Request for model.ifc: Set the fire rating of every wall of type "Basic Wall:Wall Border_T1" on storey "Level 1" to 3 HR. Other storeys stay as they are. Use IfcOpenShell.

First a look at what the model holds.

```python
import ifcopenshell
import ifcopenshell.util.element

model = ifcopenshell.open("model.ifc")
print(model.schema)
storey = next(s for s in model.by_type("IfcBuildingStorey") if s.Name == "Level 1")
walls = [e for e in ifcopenshell.util.element.get_decomposition(storey) if e.is_a("IfcWall")]
seen = {}
for e in walls:
    element_type = ifcopenshell.util.element.get_type(e)
    key = (element_type.Name if element_type != e and element_type else None, ifcopenshell.util.element.get_pset(e, "Pset_WallCommon", "FireRating"))
    seen[key] = seen.get(key, 0) + 1
for (name, value), count in sorted(seen.items(), key=str):
    print(count, "x", name, "|", value)
```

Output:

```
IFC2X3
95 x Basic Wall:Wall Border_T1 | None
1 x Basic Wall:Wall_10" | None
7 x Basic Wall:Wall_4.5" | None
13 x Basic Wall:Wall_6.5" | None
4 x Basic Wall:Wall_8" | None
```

```python
import ifcopenshell
import ifcopenshell.api.pset
import ifcopenshell.util.element

model = ifcopenshell.open("model.ifc")

storey = next(s for s in model.by_type("IfcBuildingStorey") if s.Name == "Level 1")
walls = [e for e in ifcopenshell.util.element.get_decomposition(storey) if e.is_a("IfcWall")]

count = 0
for e in walls:
    element_type = ifcopenshell.util.element.get_type(e)
    if element_type in (None, e) or element_type.Name != "Basic Wall:Wall Border_T1":
        continue
    # add_pset returns the element's existing set when there is one.
    pset = ifcopenshell.api.pset.add_pset(model, product=e, name="Pset_WallCommon")
    ifcopenshell.api.pset.edit_pset(model, pset=pset, properties={"FireRating": "3 HR"})
    count += 1

print(count, "walls updated")

model.write("model_rev.ifc")
```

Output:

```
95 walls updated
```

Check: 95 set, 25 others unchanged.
